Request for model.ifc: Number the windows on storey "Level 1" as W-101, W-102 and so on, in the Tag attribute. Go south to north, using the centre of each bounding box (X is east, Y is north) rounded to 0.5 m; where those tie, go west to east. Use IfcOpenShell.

First a look at what the model holds.

```python
import ifcopenshell
import ifcopenshell.util.element
import ifcopenshell.util.placement

model = ifcopenshell.open("model.ifc")
print(model.schema)
storey = next(s for s in model.by_type("IfcBuildingStorey") if s.Name == "Level 1")
windows = [e for e in ifcopenshell.util.element.get_decomposition(storey) if e.is_a("IfcWindow")]
for e in sorted(windows, key=lambda e: e.id()):
    origin = ifcopenshell.util.placement.get_local_placement(e.ObjectPlacement)[:3, 3]
    print(e.id(), e.Tag, e.Name, origin.round(2) + 0.0, sep=" | ")
```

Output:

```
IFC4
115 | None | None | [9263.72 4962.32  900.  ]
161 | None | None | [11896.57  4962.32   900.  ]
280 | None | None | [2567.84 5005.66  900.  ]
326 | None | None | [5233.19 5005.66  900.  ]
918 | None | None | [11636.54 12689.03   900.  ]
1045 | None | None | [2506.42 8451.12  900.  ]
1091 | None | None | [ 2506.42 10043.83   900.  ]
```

```python
import ifcopenshell
import ifcopenshell.geom
import ifcopenshell.util.element
import ifcopenshell.util.shape

model = ifcopenshell.open("model.ifc")
settings = ifcopenshell.geom.settings()
settings.set("use-world-coords", True)


def centre(element):
    shape = ifcopenshell.geom.create_shape(settings, element)
    return ifcopenshell.util.shape.get_bbox_centroid(shape.geometry)


storey = next(s for s in model.by_type("IfcBuildingStorey") if s.Name == "Level 1")
windows = [e for e in ifcopenshell.util.element.get_decomposition(storey) if e.is_a("IfcWindow")]

# Insertion points can sit at a corner or the storey origin, so sort by the geometry (in metres).
centres = {e: centre(e) for e in windows}
windows.sort(key=lambda e: (round(centres[e][1] / 0.5), centres[e][0]))

for i, e in enumerate(windows, start=1):
    number = f"W-1{i:02d}"
    e.Tag = number
    print(e.id(), number)

model.write("model_edited.ifc")
```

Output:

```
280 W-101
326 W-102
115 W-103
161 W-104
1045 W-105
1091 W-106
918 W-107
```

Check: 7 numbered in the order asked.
